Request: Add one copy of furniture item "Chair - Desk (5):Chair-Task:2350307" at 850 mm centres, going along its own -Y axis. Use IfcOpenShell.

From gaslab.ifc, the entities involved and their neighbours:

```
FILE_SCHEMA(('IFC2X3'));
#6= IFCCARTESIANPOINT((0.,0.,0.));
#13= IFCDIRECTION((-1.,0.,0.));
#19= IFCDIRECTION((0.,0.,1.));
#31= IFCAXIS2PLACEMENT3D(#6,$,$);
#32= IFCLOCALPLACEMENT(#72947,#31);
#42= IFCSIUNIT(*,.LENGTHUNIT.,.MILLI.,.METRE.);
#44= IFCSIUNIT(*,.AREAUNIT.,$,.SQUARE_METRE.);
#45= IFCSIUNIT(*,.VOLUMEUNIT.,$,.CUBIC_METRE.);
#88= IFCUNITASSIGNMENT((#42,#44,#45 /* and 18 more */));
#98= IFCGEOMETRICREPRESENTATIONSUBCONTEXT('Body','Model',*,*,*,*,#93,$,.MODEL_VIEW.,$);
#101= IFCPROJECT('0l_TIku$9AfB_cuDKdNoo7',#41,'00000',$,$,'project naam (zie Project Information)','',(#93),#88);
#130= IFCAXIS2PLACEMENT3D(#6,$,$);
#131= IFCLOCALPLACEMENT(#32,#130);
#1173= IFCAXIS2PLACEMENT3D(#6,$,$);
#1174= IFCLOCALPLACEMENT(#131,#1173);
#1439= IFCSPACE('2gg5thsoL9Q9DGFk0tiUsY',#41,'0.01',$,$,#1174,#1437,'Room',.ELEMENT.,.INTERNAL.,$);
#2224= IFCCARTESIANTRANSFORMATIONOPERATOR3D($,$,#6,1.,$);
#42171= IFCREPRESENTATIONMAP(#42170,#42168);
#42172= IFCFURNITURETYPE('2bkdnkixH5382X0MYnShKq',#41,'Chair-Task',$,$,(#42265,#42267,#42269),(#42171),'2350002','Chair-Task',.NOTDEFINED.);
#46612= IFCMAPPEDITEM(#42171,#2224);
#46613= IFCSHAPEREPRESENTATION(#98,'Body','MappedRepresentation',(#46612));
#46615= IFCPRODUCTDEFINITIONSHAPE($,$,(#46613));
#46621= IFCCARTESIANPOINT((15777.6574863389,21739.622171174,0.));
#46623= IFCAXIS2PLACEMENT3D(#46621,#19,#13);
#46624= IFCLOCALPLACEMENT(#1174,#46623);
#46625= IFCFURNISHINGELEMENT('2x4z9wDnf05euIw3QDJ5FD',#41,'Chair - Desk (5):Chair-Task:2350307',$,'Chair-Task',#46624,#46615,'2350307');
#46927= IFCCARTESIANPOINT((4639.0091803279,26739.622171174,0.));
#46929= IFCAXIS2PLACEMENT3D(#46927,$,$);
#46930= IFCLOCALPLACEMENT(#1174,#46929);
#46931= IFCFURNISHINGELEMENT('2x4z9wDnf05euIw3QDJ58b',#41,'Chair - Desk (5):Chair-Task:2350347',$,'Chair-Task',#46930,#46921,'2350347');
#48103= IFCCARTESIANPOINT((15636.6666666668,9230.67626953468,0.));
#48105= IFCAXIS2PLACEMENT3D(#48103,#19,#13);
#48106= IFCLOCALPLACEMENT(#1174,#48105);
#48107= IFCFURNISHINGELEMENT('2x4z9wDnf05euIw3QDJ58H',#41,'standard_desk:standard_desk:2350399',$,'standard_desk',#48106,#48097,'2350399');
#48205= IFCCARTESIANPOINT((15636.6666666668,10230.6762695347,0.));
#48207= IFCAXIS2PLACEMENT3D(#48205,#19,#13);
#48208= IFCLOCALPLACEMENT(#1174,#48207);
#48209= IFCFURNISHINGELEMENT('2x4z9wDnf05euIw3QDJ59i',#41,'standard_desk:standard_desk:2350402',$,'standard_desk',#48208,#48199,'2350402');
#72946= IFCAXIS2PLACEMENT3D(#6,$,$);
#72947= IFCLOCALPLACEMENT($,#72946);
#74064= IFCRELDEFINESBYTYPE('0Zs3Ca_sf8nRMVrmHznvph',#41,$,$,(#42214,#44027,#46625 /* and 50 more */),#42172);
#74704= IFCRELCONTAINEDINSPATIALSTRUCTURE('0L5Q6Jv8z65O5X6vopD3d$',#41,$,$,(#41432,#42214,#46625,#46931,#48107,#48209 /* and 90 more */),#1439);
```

```python
import ifcopenshell
import ifcopenshell.api.geometry
import ifcopenshell.api.root
import ifcopenshell.util.element
import ifcopenshell.util.placement

model = ifcopenshell.open("gaslab.ifc")


def reuse_history(source, copy):
    """copy_class also copies each property set's owner history, people and application; keep the originals."""
    for rel in copy.IsDefinedBy:
        if rel.is_a("IfcRelDefinesByProperties") and (history := rel.RelatingPropertyDefinition.OwnerHistory):
            rel.RelatingPropertyDefinition.OwnerHistory = source.OwnerHistory
            ifcopenshell.util.element.remove_deep2(model, history)


source = model.by_id(46625)
base = ifcopenshell.util.placement.get_local_placement(source.ObjectPlacement)
step = -base[:3, 1] * 850.0

for i in range(1, 2):
    copy = ifcopenshell.api.root.copy_class(model, product=source)
    copy.Representation = ifcopenshell.util.element.copy_deep(
        model, source.Representation, exclude=["IfcGeometricRepresentationContext", "IfcRepresentationMap"]
    )
    copy.Name = "Chair - Desk (5):Chair-Task"
    copy.Tag = None
    reuse_history(source, copy)
    matrix = base.copy()
    matrix[:3, 3] += i * step
    print("added at", matrix[:3, 3].round(3) + 0.0)
    ifcopenshell.api.geometry.edit_object_placement(model, product=copy, matrix=matrix, is_si=False)

model.write("gaslab_v2.ifc")
```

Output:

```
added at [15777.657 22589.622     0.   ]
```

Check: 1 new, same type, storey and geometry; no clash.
